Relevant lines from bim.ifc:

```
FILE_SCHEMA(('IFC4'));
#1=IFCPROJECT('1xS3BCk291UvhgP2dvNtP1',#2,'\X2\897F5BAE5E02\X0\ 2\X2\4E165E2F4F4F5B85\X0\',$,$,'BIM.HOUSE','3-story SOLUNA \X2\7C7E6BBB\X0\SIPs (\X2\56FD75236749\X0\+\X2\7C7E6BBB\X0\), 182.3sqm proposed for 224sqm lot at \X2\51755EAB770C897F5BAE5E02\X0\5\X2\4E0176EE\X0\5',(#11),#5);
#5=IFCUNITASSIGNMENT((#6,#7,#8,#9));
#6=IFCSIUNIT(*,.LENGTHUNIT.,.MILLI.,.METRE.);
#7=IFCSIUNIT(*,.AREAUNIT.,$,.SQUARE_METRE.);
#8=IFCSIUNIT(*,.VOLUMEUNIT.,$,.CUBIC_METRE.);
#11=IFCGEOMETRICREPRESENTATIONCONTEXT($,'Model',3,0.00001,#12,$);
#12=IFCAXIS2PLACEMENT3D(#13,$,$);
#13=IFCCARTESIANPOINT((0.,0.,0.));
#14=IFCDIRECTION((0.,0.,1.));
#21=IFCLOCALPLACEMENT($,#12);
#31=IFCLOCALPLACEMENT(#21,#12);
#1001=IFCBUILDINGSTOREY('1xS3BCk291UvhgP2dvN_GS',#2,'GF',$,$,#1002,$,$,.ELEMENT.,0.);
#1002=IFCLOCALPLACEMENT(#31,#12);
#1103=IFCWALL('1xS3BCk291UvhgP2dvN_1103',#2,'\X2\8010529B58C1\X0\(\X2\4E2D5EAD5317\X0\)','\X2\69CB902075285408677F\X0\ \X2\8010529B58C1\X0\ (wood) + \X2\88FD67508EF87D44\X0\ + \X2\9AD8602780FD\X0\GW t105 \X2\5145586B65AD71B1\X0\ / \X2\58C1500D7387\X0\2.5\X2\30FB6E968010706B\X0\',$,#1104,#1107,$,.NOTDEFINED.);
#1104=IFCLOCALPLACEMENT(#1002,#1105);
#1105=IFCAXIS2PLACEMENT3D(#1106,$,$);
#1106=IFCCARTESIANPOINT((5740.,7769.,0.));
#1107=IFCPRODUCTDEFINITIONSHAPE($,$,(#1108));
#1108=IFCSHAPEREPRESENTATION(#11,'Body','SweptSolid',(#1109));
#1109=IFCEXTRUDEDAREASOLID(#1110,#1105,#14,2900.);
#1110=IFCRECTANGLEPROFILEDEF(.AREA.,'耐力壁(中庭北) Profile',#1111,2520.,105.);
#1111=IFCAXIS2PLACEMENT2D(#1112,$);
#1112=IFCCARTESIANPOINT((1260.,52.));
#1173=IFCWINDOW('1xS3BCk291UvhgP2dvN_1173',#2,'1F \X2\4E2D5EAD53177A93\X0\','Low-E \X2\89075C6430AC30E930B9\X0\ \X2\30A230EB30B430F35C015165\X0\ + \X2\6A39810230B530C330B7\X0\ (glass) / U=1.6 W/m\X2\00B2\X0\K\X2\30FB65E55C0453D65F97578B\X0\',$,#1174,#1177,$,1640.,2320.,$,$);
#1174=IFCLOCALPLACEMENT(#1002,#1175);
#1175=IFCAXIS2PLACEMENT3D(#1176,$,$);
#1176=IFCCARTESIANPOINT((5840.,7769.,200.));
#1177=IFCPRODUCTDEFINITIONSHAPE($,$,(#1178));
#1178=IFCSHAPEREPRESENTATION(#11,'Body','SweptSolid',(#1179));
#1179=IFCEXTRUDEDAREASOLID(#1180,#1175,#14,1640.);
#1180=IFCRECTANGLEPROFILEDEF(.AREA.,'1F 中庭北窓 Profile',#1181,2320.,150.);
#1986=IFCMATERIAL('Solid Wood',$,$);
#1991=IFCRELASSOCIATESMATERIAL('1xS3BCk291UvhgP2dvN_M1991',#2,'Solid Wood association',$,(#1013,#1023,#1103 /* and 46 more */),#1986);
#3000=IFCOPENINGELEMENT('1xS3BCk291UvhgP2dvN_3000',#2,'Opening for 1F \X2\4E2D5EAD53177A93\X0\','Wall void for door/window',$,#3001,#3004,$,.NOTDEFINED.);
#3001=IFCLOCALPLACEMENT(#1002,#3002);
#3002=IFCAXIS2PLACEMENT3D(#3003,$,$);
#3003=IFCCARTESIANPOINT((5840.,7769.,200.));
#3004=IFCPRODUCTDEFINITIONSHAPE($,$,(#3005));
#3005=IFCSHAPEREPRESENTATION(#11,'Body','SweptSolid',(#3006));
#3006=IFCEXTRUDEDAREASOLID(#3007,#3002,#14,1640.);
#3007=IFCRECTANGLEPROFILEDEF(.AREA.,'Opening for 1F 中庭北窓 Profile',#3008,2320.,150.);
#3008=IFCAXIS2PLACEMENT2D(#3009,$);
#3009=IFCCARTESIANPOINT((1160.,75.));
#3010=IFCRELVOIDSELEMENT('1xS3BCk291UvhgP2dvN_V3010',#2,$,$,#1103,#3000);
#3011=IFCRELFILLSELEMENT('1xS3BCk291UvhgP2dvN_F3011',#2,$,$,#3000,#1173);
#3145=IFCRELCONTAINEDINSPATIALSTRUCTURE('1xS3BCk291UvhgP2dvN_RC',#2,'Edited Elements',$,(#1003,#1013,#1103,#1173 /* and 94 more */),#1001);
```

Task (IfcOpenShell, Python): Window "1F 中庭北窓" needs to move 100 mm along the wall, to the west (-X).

```python
import ifcopenshell
import ifcopenshell.api.geometry
import ifcopenshell.util.placement

model = ifcopenshell.open("bim.ifc")

window = model.by_id(1173)
opening = window.FillsVoids[0].RelatingOpeningElement
wall = opening.VoidsElements[0].RelatingBuildingElement

wall_matrix = ifcopenshell.util.placement.get_local_placement(wall.ObjectPlacement)
shift = wall_matrix[:3, 0] * -100.0
before = ifcopenshell.util.placement.get_local_placement(window.ObjectPlacement)[:3, 3].copy()

# The window is not placed relative to its opening, so move both.
for product in (opening, window):
    matrix = ifcopenshell.util.placement.get_local_placement(product.ObjectPlacement)
    matrix[:3, 3] += shift
    ifcopenshell.api.geometry.edit_object_placement(model, product=product, matrix=matrix, is_si=False)

after = ifcopenshell.util.placement.get_local_placement(window.ObjectPlacement)[:3, 3]
print("window moved by", (after - before).round(3) + 0.0)

model.write("bim_edited.ifc")
```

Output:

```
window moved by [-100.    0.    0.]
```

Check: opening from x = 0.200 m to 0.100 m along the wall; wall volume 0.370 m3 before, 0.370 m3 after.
